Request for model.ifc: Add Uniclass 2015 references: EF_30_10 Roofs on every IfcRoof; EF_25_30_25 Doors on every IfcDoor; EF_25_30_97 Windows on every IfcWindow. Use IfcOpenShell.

First a look at what the model holds.

```python
import ifcopenshell

model = ifcopenshell.open("model.ifc")
print(model.schema)
print("classifications:", [c.Name for c in model.by_type("IfcClassification")])
for ifc_class in ("IfcDoor", "IfcRoof", "IfcStair", "IfcWall", "IfcWindow"):
    print(ifc_class, len(model.by_type(ifc_class)))
```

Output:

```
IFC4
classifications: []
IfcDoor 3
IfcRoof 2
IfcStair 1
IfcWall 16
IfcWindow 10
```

```python
import ifcopenshell
import ifcopenshell.api.classification

model = ifcopenshell.open("model.ifc")

system = ifcopenshell.api.classification.add_classification(model, classification="Uniclass 2015")

codes = {
    "IfcRoof": ("EF_30_10", "Roofs"),
    "IfcDoor": ("EF_25_30_25", "Doors"),
    "IfcWindow": ("EF_25_30_97", "Windows"),
}
for ifc_class, (code, name) in codes.items():
    products = model.by_type(ifc_class)
    ifcopenshell.api.classification.add_reference(
        model, products=products, classification=system, identification=code, name=name
    )
    print(code, len(products))

model.write("model_rev.ifc")
```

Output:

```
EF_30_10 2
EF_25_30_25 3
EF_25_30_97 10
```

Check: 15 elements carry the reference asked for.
